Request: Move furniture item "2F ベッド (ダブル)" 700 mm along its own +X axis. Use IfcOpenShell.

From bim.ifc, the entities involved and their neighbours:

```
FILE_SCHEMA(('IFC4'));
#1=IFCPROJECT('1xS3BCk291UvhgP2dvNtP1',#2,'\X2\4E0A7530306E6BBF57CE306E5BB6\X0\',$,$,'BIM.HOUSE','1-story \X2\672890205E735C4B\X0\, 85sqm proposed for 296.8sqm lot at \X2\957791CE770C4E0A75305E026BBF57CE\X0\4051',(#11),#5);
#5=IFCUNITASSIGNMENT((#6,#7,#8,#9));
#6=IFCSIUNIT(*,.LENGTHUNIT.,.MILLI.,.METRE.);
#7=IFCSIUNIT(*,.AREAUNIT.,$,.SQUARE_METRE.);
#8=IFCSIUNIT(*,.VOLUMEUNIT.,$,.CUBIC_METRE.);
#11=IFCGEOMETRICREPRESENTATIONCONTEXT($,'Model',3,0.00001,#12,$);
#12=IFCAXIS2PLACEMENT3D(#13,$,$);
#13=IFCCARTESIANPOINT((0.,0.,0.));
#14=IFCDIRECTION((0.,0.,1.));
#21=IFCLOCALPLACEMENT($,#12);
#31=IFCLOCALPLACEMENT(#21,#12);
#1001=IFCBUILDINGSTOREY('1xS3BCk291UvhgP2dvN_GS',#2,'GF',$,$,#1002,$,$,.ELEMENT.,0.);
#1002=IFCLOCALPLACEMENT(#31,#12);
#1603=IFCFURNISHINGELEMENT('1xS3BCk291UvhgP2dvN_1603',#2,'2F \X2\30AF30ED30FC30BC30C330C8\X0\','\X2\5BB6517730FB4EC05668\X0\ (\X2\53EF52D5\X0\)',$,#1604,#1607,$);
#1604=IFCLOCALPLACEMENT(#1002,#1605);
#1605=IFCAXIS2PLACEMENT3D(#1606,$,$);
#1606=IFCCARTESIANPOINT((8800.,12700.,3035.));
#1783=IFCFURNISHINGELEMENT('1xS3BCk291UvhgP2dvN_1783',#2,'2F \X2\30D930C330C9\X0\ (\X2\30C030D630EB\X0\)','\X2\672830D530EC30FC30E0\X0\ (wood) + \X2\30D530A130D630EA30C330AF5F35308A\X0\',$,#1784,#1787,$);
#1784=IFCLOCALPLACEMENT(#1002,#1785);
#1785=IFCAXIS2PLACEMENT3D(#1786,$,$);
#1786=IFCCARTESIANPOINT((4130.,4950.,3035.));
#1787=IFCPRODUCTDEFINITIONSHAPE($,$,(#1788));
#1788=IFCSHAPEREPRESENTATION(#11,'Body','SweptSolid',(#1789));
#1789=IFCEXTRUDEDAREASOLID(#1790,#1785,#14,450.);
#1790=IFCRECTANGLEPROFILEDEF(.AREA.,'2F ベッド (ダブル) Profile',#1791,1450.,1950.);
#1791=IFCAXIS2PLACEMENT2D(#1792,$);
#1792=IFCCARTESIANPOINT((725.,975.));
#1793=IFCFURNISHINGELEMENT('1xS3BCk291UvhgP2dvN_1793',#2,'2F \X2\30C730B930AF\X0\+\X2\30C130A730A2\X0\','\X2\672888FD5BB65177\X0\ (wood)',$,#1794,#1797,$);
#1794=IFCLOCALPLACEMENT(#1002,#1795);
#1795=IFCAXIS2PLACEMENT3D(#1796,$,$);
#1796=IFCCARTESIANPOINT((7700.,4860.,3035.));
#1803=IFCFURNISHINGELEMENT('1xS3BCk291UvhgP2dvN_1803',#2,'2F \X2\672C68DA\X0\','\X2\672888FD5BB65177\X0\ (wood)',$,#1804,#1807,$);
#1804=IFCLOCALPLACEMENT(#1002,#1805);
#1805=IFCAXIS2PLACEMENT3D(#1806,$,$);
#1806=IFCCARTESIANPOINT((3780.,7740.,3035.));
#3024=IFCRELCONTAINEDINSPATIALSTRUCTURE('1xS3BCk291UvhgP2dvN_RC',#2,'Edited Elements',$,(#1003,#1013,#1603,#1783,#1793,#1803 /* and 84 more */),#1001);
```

```python
import ifcopenshell
import ifcopenshell.api.geometry
import ifcopenshell.util.placement
import ifcopenshell.util.unit

model = ifcopenshell.open("bim.ifc")
unit_scale = ifcopenshell.util.unit.calculate_unit_scale(model)

item = model.by_id(1783)
matrix = ifcopenshell.util.placement.get_local_placement(item.ObjectPlacement)
matrix[:3, 3] += matrix[:3, 0] * 0.7 / unit_scale
ifcopenshell.api.geometry.edit_object_placement(model, product=item, matrix=matrix, is_si=False)

print(ifcopenshell.util.placement.get_local_placement(item.ObjectPlacement).round(3) + 0.0)

model.write("bim_v2.ifc")
```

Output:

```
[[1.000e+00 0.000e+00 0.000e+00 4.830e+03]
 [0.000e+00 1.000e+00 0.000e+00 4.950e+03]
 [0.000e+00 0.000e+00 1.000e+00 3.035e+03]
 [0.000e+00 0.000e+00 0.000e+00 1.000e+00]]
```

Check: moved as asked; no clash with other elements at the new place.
